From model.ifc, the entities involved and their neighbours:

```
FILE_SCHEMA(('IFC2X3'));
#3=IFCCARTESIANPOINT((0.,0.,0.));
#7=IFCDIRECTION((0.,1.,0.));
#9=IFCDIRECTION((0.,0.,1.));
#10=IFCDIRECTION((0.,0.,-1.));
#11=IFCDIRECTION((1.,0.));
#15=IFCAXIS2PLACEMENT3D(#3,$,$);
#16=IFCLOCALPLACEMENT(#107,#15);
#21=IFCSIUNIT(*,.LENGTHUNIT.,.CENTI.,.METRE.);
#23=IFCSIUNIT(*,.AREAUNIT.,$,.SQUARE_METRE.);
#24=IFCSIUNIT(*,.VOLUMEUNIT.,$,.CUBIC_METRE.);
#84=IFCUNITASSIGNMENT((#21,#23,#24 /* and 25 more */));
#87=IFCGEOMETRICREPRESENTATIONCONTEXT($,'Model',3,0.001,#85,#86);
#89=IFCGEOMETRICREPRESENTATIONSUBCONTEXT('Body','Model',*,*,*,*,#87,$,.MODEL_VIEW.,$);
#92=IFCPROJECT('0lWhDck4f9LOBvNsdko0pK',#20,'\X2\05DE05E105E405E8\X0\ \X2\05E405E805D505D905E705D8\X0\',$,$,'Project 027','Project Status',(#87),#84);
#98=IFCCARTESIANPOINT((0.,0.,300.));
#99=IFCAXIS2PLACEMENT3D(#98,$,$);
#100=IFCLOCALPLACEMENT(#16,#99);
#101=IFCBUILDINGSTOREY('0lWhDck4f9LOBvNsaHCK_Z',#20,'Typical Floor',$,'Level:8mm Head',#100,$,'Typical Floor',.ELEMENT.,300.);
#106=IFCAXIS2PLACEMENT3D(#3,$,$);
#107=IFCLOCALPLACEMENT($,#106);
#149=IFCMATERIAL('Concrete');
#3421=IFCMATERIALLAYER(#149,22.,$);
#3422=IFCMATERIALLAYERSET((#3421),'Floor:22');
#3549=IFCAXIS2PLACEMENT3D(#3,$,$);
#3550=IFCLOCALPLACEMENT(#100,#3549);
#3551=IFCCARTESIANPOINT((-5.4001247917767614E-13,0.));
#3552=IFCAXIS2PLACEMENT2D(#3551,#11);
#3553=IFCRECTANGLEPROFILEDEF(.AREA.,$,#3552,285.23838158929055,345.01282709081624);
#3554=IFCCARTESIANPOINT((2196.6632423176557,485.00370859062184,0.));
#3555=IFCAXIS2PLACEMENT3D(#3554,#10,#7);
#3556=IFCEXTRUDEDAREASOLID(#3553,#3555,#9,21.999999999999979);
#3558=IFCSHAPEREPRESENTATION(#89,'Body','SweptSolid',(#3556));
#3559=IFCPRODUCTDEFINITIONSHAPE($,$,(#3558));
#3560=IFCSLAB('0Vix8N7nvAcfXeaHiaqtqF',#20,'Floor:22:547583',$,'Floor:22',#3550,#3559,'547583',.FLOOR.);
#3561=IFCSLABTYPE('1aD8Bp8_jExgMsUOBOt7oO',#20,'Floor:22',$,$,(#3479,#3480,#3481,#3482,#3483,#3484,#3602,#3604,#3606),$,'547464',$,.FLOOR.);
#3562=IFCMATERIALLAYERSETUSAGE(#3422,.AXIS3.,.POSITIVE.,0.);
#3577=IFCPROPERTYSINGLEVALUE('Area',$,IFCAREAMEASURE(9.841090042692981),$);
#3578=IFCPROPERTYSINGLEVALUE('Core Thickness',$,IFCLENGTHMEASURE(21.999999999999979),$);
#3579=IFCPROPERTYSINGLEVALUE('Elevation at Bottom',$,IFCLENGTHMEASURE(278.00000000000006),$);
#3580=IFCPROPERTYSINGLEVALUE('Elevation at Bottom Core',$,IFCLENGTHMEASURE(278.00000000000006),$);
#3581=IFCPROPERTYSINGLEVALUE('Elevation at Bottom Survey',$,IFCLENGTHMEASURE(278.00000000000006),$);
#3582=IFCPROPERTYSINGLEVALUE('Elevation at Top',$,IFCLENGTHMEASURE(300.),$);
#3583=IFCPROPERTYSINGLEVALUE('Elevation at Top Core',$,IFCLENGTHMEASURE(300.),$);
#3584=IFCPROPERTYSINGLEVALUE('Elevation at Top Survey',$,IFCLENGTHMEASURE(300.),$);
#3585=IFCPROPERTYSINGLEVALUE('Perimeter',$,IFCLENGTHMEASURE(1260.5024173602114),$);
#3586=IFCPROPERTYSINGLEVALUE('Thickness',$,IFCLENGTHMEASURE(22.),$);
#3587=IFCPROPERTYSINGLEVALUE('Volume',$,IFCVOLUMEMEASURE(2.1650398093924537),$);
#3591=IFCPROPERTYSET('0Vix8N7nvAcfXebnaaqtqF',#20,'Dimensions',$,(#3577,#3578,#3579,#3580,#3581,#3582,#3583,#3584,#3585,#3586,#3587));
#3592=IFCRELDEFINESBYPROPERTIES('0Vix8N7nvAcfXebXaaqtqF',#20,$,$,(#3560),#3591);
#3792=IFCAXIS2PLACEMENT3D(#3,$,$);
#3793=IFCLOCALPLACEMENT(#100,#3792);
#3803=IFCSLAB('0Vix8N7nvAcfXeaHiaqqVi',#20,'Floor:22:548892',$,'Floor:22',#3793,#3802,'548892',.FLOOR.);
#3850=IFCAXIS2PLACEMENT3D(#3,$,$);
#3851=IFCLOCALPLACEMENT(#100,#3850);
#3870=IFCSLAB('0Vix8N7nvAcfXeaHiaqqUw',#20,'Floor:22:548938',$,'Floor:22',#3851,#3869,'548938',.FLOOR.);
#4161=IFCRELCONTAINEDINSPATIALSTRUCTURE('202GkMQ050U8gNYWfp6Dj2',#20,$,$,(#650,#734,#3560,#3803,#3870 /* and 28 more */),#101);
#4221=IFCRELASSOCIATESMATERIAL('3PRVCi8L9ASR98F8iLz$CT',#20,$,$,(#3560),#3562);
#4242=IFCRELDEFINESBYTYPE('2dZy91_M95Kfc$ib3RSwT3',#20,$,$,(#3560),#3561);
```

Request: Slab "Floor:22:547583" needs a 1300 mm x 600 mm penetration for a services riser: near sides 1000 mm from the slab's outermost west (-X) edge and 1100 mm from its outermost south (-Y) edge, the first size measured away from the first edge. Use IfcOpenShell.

```python
import numpy as np
import ifcopenshell
import ifcopenshell.api.feature
import ifcopenshell.api.geometry
import ifcopenshell.api.pset
import ifcopenshell.api.root
import ifcopenshell.geom
import ifcopenshell.util.element
import ifcopenshell.util.placement
import ifcopenshell.util.representation
import ifcopenshell.util.shape
import ifcopenshell.util.unit

model = ifcopenshell.open("model.ifc")
unit_scale = ifcopenshell.util.unit.calculate_unit_scale(model)
area_scale = ifcopenshell.util.unit.calculate_unit_scale(model, "AREAUNIT")
volume_scale = ifcopenshell.util.unit.calculate_unit_scale(model, "VOLUMEUNIT")
settings = ifcopenshell.geom.settings()


def volume(element):
    """Net volume in cubic metres, openings subtracted."""
    shape = ifcopenshell.geom.create_shape(settings, element)
    return ifcopenshell.util.shape.get_volume(shape.geometry)


slab = model.by_guid("0Vix8N7nvAcfXeaHiaqtqF")
before = volume(slab)

# Extent in the slab's own axes, in metres. The edges named are its -X and -Y sides.
slab_shape = ifcopenshell.geom.create_shape(settings, slab)
vertices = ifcopenshell.util.shape.get_vertices(slab_shape.geometry)
x_min, y_min, bottom = vertices.min(axis=0)
top = vertices[:, 2].max()

opening = ifcopenshell.api.root.create_entity(model, ifc_class="IfcOpeningElement", name="Services riser opening")
context = ifcopenshell.util.representation.get_context(model, "Model", "Body", "MODEL_VIEW")
width, depth = 1.3, 0.6
outline = [(0.0, 0.0), (width, 0.0), (width, depth), (0.0, depth), (0.0, 0.0)]
# Overshoot both faces by 50 mm so the cut is clean.
shape = ifcopenshell.api.geometry.add_slab_representation(
    model, context=context, depth=top - bottom + 0.1, polyline=outline
)
ifcopenshell.api.geometry.assign_representation(model, product=opening, representation=shape)

matrix = ifcopenshell.util.placement.get_local_placement(slab.ObjectPlacement)
matrix[:, 3] = matrix @ np.append(np.array([x_min + 1, y_min + 1.1, bottom - 0.05]) / unit_scale, 1.0)
ifcopenshell.api.geometry.edit_object_placement(model, product=opening, matrix=matrix, is_si=False)
ifcopenshell.api.feature.add_feature(model, feature=opening, element=slab)

after = volume(slab)

# Update the slab's stored quantities.
pset = model.by_id(ifcopenshell.util.element.get_pset(slab, "Dimensions", should_inherit=False)["id"])
ifcopenshell.api.pset.edit_pset(model, pset=pset, properties={
    "Area": model.create_entity("IfcAreaMeasure", after / (top - bottom) / area_scale),
    "Volume": model.create_entity("IfcVolumeMeasure", after / volume_scale),
})

print(f"slab volume {before:.3f} -> {after:.3f} m3")

model.write("model_updated.ifc")
```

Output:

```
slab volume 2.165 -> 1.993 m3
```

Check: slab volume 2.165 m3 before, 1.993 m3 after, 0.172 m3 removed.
